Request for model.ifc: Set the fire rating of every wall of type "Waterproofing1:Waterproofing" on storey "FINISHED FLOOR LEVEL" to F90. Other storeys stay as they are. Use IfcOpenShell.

First a look at what the model holds.

```python
import ifcopenshell
import ifcopenshell.util.element

model = ifcopenshell.open("model.ifc")
print(model.schema)
storey = next(s for s in model.by_type("IfcBuildingStorey") if s.Name == "FINISHED FLOOR LEVEL")
walls = [e for e in ifcopenshell.util.element.get_decomposition(storey) if e.is_a("IfcWall")]
seen = {}
for e in walls:
    element_type = ifcopenshell.util.element.get_type(e)
    key = (element_type.Name if element_type != e and element_type else None, ifcopenshell.util.element.get_pset(e, "Pset_WallCommon", "FireRating"))
    seen[key] = seen.get(key, 0) + 1
for (name, value), count in sorted(seen.items(), key=str):
    print(count, "x", name, "|", value)
```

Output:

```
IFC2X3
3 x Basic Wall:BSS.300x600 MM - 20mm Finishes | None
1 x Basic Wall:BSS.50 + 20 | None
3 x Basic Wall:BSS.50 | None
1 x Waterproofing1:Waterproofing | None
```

```python
import ifcopenshell
import ifcopenshell.api.pset
import ifcopenshell.util.element

model = ifcopenshell.open("model.ifc")

storey = next(s for s in model.by_type("IfcBuildingStorey") if s.Name == "FINISHED FLOOR LEVEL")
walls = [e for e in ifcopenshell.util.element.get_decomposition(storey) if e.is_a("IfcWall")]

count = 0
for e in walls:
    element_type = ifcopenshell.util.element.get_type(e)
    if element_type in (None, e) or element_type.Name != "Waterproofing1:Waterproofing":
        continue
    # add_pset returns the element's existing set when there is one.
    pset = ifcopenshell.api.pset.add_pset(model, product=e, name="Pset_WallCommon")
    ifcopenshell.api.pset.edit_pset(model, pset=pset, properties={"FireRating": "F90"})
    count += 1

print(count, "walls updated")

model.write("model-out.ifc")
```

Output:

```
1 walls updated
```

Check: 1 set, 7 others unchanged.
